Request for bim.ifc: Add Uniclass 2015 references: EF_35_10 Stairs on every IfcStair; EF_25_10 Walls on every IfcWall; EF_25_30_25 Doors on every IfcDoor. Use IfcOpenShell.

First a look at what the model holds.

```python
import ifcopenshell

model = ifcopenshell.open("bim.ifc")
print(model.schema)
print("classifications:", [c.Name for c in model.by_type("IfcClassification")])
for ifc_class in ("IfcDoor", "IfcRoof", "IfcStair", "IfcWall", "IfcWindow"):
    print(ifc_class, len(model.by_type(ifc_class)))
```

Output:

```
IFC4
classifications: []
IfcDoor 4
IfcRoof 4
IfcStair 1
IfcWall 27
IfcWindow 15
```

```python
import ifcopenshell
import ifcopenshell.api.classification

model = ifcopenshell.open("bim.ifc")

system = ifcopenshell.api.classification.add_classification(model, classification="Uniclass 2015")

codes = {
    "IfcStair": ("EF_35_10", "Stairs"),
    "IfcWall": ("EF_25_10", "Walls"),
    "IfcDoor": ("EF_25_30_25", "Doors"),
}
for ifc_class, (code, name) in codes.items():
    products = model.by_type(ifc_class)
    ifcopenshell.api.classification.add_reference(
        model, products=products, classification=system, identification=code, name=name
    )
    print(code, len(products))

model.write("bim_rev.ifc")
```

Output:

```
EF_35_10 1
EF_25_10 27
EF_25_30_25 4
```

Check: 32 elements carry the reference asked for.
